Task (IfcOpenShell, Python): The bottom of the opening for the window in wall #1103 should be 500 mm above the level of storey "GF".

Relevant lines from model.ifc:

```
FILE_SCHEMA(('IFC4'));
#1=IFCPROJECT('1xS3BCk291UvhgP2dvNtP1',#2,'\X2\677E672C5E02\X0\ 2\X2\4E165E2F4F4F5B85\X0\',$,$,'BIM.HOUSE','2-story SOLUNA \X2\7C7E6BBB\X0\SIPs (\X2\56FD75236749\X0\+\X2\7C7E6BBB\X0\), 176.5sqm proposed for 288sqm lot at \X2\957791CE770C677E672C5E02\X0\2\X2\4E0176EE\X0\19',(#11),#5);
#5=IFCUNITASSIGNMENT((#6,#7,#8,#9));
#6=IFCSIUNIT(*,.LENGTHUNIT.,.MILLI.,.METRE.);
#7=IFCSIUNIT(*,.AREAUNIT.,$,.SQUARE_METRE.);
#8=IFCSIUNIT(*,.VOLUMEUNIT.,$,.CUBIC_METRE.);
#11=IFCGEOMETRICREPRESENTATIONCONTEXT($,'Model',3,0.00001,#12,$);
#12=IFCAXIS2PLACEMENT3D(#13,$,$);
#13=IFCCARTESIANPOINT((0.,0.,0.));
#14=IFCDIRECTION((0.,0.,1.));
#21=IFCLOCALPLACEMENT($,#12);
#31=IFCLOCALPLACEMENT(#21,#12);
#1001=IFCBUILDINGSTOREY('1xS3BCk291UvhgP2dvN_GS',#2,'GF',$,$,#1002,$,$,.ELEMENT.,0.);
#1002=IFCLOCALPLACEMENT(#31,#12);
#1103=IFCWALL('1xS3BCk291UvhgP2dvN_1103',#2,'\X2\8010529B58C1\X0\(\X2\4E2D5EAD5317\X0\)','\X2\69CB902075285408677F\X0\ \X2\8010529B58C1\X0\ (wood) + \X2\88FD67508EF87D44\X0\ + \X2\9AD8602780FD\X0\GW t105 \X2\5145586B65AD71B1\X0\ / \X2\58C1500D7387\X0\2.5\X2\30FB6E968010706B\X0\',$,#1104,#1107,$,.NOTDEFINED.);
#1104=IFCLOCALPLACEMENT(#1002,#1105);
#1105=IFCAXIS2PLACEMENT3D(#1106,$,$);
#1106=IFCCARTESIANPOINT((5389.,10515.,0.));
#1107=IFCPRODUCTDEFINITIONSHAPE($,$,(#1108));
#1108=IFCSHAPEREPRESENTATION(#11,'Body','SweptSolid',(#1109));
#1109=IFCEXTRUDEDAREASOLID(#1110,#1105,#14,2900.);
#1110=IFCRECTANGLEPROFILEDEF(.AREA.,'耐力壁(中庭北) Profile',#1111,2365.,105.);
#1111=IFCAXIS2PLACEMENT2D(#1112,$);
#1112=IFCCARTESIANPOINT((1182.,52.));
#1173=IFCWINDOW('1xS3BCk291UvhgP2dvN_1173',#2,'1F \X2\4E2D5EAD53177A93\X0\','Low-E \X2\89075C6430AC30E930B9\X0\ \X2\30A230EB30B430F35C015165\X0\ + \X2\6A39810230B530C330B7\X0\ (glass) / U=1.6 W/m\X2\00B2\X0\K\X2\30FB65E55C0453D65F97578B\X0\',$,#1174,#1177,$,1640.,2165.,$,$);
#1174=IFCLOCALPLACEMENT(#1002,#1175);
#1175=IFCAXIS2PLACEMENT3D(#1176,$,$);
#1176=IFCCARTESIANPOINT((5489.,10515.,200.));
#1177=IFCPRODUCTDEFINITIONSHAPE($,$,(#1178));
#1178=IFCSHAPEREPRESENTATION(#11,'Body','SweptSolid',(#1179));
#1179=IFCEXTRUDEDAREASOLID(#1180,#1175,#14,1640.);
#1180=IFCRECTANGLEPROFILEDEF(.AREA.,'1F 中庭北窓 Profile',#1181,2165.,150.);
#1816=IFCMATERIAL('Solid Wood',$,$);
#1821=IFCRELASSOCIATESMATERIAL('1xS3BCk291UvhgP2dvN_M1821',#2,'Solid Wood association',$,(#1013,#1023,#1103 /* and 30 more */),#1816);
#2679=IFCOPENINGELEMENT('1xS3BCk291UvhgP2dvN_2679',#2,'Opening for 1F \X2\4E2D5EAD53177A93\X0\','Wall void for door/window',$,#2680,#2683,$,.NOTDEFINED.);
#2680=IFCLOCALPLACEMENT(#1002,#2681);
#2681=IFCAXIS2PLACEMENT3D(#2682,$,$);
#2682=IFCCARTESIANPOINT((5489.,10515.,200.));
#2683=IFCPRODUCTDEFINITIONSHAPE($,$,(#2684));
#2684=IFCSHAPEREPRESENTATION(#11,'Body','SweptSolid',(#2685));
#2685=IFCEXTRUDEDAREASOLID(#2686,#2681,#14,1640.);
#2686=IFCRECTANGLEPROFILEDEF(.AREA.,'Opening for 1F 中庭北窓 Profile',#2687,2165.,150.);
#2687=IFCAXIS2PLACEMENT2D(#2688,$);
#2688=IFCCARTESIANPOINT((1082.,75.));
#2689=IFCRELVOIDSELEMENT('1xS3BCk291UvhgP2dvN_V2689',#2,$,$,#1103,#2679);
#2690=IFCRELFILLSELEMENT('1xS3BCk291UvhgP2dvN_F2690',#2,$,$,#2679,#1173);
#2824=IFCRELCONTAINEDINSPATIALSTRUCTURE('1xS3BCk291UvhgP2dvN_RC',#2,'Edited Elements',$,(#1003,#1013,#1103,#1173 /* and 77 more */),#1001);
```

```python
import numpy as np
import ifcopenshell
import ifcopenshell.api.geometry
import ifcopenshell.geom
import ifcopenshell.util.element
import ifcopenshell.util.placement
import ifcopenshell.util.shape
import ifcopenshell.util.unit

model = ifcopenshell.open("model.ifc")
unit_scale = ifcopenshell.util.unit.calculate_unit_scale(model)

window = model.by_guid("1xS3BCk291UvhgP2dvN_1173")
opening = window.FillsVoids[0].RelatingOpeningElement
storey = ifcopenshell.util.element.get_container(window, ifc_class="IfcBuildingStorey")
level = ifcopenshell.util.placement.get_local_placement(storey.ObjectPlacement)[2, 3]

# The opening's origin need not be at the sill, so measure its lowest point.
shape = ifcopenshell.geom.create_shape(ifcopenshell.geom.settings(), opening)
bottom = ifcopenshell.util.shape.get_shape_bottom_elevation(shape, shape.geometry) / unit_scale
dz = level + 500.0 - bottom

shift = np.array([0.0, 0.0, dz])
# The window is not placed relative to its opening, so move both.
for product in (opening, window):
    matrix = ifcopenshell.util.placement.get_local_placement(product.ObjectPlacement)
    matrix[:3, 3] += shift
    ifcopenshell.api.geometry.edit_object_placement(model, product=product, matrix=matrix, is_si=False)

print(f"moved by {dz * unit_scale:+.3f} m")

model.write("model-out.ifc")
```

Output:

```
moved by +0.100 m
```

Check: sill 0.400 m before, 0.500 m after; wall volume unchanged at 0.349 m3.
